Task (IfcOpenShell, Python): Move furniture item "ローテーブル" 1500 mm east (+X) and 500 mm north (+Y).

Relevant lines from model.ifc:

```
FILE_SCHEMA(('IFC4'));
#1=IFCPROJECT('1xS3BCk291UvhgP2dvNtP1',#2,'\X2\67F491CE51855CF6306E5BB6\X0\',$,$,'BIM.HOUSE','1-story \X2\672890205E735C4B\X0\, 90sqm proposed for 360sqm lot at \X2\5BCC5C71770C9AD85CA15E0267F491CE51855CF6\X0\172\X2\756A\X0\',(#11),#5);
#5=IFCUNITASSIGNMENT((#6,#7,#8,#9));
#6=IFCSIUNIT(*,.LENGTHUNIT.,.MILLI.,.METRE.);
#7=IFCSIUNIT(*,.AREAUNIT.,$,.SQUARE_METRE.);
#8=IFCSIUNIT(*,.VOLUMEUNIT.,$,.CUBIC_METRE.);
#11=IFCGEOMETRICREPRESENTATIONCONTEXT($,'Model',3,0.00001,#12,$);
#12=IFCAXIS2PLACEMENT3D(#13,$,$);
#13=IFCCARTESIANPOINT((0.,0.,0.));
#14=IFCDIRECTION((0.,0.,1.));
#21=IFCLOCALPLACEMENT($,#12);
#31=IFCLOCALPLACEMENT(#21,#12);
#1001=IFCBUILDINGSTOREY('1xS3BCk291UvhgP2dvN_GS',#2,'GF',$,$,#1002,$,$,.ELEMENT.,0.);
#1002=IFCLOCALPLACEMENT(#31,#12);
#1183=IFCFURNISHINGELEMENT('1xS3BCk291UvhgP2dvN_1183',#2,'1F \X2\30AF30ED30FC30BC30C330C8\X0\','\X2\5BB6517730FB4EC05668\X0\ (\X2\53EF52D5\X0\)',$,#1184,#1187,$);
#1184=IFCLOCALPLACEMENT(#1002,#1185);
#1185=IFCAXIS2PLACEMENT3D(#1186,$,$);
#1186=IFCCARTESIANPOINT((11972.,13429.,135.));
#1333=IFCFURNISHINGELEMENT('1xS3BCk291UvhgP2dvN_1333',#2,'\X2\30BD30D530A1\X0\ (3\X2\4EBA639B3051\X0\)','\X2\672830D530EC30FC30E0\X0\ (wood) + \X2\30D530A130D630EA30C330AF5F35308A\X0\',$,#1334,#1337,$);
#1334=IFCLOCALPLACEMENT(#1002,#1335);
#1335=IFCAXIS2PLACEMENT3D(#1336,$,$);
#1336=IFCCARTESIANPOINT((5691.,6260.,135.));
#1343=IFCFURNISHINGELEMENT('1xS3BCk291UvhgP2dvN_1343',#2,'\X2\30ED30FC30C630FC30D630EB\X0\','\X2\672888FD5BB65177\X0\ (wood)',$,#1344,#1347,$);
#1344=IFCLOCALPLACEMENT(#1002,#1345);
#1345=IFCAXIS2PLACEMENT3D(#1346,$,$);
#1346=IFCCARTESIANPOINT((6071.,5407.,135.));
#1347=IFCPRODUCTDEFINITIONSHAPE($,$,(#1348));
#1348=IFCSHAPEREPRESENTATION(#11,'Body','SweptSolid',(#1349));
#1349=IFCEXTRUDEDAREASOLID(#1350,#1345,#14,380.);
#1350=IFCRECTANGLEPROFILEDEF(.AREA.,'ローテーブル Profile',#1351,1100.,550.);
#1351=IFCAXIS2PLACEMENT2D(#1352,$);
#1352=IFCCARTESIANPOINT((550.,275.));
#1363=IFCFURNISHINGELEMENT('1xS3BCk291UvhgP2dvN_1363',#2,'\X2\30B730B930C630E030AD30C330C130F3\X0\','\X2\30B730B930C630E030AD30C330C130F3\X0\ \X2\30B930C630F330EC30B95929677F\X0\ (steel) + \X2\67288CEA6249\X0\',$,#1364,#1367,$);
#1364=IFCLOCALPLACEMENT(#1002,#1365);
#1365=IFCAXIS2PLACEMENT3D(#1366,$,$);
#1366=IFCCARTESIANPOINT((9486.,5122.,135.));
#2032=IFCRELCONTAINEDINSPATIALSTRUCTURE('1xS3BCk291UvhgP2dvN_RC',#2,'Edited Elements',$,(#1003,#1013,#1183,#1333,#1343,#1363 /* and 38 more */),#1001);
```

```python
import ifcopenshell
import ifcopenshell.api.geometry
import ifcopenshell.util.placement
import ifcopenshell.util.unit

model = ifcopenshell.open("model.ifc")
unit_scale = ifcopenshell.util.unit.calculate_unit_scale(model)

item = model.by_guid("1xS3BCk291UvhgP2dvN_1343")
matrix = ifcopenshell.util.placement.get_local_placement(item.ObjectPlacement)
matrix[0, 3] += 1.5 / unit_scale
matrix[1, 3] += 0.5 / unit_scale
ifcopenshell.api.geometry.edit_object_placement(model, product=item, matrix=matrix, is_si=False)

print(ifcopenshell.util.placement.get_local_placement(item.ObjectPlacement).round(3) + 0.0)

model.write("model-out.ifc")
```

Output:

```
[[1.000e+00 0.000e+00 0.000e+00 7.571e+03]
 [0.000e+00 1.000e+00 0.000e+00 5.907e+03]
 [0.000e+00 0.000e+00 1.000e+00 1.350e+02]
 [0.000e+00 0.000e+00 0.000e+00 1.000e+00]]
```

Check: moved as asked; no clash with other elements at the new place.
